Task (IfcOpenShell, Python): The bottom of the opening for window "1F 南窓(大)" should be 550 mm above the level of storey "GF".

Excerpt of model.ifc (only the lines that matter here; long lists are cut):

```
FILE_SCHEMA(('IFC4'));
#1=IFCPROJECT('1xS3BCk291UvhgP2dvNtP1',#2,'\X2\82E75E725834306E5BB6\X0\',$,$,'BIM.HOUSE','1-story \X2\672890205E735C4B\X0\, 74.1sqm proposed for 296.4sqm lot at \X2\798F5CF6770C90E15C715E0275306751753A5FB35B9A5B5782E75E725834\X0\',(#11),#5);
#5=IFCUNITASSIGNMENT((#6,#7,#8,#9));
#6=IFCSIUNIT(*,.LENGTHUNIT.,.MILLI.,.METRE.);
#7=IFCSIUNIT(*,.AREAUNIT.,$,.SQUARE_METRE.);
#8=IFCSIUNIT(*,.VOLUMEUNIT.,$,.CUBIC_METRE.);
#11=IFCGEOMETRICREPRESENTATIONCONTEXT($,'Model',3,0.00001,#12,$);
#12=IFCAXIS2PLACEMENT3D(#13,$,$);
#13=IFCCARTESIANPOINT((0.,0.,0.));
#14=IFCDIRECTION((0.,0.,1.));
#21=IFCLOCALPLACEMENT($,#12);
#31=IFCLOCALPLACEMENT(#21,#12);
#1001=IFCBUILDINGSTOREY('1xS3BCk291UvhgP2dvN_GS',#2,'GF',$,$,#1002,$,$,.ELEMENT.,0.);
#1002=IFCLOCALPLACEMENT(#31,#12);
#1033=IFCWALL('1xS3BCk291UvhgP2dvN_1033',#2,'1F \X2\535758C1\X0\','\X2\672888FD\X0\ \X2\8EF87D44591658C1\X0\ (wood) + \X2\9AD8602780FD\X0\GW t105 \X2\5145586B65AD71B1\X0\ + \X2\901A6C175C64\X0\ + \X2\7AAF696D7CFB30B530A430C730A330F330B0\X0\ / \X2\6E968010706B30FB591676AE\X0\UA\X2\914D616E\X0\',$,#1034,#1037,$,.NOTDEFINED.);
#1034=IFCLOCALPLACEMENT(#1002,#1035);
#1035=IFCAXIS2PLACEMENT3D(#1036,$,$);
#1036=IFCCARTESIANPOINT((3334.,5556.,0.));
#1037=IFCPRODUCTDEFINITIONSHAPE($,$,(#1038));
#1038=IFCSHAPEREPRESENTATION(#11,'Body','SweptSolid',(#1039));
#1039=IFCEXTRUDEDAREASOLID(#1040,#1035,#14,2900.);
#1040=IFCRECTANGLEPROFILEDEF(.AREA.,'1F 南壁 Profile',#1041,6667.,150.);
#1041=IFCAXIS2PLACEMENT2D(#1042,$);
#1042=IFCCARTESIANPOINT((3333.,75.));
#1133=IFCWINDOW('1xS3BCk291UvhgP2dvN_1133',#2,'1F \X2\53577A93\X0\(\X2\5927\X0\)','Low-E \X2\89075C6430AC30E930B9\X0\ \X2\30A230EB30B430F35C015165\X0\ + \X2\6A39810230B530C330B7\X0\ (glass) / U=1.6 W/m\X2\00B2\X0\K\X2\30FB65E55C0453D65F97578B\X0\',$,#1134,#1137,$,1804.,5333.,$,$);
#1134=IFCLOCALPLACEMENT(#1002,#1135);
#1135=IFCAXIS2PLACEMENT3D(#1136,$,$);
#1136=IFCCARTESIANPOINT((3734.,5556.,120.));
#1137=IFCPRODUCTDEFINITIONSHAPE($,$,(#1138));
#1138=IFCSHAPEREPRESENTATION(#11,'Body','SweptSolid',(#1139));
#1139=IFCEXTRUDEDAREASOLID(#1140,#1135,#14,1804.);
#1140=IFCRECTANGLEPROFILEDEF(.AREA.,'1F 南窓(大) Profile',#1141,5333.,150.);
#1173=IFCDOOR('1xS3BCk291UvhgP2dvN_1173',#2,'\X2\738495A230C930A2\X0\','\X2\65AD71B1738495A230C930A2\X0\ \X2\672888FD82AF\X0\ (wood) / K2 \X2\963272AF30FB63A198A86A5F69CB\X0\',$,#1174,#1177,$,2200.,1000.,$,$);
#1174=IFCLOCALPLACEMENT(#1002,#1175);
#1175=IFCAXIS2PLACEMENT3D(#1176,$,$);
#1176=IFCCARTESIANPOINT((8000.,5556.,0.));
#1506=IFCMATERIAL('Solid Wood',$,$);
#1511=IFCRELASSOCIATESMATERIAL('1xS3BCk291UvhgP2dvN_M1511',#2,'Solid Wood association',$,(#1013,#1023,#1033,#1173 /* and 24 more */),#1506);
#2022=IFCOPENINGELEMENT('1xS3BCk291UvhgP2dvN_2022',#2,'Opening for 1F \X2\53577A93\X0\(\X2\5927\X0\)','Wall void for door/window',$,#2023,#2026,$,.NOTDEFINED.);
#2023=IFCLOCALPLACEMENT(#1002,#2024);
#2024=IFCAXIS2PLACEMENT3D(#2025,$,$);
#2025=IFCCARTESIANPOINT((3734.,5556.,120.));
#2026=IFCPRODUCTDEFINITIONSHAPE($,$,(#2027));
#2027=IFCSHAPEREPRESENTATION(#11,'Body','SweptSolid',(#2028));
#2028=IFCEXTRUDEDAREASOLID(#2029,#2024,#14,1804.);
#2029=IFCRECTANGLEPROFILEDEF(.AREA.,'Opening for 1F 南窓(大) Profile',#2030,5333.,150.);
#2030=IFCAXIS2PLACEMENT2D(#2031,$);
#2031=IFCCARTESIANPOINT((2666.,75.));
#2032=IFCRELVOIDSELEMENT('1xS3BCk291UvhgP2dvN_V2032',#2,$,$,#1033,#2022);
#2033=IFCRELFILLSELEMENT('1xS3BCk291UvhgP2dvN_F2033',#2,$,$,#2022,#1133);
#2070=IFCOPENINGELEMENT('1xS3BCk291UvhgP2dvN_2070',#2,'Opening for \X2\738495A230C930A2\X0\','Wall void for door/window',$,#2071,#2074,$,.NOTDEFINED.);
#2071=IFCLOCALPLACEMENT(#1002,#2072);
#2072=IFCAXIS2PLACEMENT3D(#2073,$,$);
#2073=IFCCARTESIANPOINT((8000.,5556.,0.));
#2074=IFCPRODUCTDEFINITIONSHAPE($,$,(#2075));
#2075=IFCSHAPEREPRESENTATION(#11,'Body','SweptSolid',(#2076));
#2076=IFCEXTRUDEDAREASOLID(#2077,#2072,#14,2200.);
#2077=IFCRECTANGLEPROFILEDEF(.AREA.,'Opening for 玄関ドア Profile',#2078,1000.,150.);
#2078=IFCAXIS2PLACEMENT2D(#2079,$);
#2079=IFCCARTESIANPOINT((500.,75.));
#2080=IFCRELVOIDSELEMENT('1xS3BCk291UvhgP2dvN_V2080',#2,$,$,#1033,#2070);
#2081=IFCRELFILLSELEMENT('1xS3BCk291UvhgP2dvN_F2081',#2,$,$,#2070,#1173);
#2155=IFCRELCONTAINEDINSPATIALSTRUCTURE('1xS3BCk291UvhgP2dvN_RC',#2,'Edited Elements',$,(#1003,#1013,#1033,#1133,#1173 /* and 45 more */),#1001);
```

```python
import numpy as np
import ifcopenshell
import ifcopenshell.api.geometry
import ifcopenshell.geom
import ifcopenshell.util.element
import ifcopenshell.util.placement
import ifcopenshell.util.shape
import ifcopenshell.util.unit

model = ifcopenshell.open("model.ifc")
unit_scale = ifcopenshell.util.unit.calculate_unit_scale(model)

window = model.by_id(1133)
opening = window.FillsVoids[0].RelatingOpeningElement
storey = ifcopenshell.util.element.get_container(window, ifc_class="IfcBuildingStorey")
level = ifcopenshell.util.placement.get_local_placement(storey.ObjectPlacement)[2, 3]

# The opening's origin need not be at the sill, so measure its lowest point.
shape = ifcopenshell.geom.create_shape(ifcopenshell.geom.settings(), opening)
bottom = ifcopenshell.util.shape.get_shape_bottom_elevation(shape, shape.geometry) / unit_scale
dz = level + 0.55 / unit_scale - bottom

shift = np.array([0.0, 0.0, dz])
# The window is not placed relative to its opening, so move both.
for product in (opening, window):
    matrix = ifcopenshell.util.placement.get_local_placement(product.ObjectPlacement)
    matrix[:3, 3] += shift
    ifcopenshell.api.geometry.edit_object_placement(model, product=product, matrix=matrix, is_si=False)

print(f"moved by {dz * unit_scale:+.3f} m")

model.write("model_edited.ifc")
```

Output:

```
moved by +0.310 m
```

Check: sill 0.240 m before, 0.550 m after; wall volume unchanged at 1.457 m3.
